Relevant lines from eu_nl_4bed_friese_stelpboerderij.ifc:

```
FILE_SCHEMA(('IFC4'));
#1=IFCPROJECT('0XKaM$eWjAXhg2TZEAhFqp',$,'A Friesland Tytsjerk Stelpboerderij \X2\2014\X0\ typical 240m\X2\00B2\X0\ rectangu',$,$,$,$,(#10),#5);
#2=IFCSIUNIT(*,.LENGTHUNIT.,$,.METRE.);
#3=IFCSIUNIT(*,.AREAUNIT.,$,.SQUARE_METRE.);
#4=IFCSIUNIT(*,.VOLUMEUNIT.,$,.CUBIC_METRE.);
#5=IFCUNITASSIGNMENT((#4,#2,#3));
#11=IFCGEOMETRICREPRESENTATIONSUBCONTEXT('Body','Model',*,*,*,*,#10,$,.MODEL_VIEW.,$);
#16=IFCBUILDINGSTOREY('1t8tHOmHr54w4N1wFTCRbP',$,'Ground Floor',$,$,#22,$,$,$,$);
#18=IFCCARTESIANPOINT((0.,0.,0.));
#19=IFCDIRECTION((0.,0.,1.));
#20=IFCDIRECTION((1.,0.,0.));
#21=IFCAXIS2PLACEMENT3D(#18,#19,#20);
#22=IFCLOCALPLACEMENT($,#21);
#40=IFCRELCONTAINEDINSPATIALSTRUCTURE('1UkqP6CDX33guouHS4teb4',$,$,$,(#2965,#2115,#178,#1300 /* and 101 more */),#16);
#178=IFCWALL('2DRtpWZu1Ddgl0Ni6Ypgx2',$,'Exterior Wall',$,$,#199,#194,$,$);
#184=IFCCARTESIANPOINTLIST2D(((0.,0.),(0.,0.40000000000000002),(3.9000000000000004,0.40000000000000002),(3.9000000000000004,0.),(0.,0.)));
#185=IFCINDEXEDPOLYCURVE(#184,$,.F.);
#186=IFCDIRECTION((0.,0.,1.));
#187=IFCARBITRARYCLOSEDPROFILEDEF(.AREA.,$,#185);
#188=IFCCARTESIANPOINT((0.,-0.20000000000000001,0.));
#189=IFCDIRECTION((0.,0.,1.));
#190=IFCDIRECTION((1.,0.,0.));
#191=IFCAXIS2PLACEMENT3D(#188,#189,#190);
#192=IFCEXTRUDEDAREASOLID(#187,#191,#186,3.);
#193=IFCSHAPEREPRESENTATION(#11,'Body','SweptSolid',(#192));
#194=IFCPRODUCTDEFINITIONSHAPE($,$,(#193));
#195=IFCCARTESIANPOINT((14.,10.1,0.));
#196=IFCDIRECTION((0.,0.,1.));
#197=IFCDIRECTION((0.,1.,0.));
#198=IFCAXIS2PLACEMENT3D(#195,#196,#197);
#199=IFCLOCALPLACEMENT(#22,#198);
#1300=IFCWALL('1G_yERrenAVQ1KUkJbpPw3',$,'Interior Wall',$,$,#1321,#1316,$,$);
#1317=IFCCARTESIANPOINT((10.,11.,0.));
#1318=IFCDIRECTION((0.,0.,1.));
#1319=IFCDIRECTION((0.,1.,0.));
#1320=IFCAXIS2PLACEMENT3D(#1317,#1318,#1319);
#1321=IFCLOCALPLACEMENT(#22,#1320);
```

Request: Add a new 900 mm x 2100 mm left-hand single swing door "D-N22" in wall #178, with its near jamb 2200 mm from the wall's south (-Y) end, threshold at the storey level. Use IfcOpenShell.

```python
import numpy as np
import ifcopenshell
import ifcopenshell.api.feature
import ifcopenshell.api.geometry
import ifcopenshell.api.root
import ifcopenshell.api.spatial
import ifcopenshell.geom
import ifcopenshell.util.element
import ifcopenshell.util.placement
import ifcopenshell.util.representation
import ifcopenshell.util.shape
import ifcopenshell.util.unit

model = ifcopenshell.open("eu_nl_4bed_friese_stelpboerderij.ifc")
unit_scale = ifcopenshell.util.unit.calculate_unit_scale(model)
settings = ifcopenshell.geom.settings()


def volume(element):
    """Net volume in cubic metres, openings subtracted."""
    shape = ifcopenshell.geom.create_shape(settings, element)
    return ifcopenshell.util.shape.get_volume(shape.geometry)


wall = model.by_guid("2DRtpWZu1Ddgl0Ni6Ypgx2")
storey = ifcopenshell.util.element.get_container(wall, ifc_class="IfcBuildingStorey")
context = ifcopenshell.util.representation.get_context(model, "Model", "Body", "MODEL_VIEW")
before = volume(wall)

width, height, from_end, sill = 0.9, 2.1, 2.2, 0.0  # metres

# The wall runs along its own X axis, and the end named is its -X end.
wall_shape = ifcopenshell.geom.create_shape(settings, wall)
x, y, z = ifcopenshell.util.shape.get_vertices(wall_shape.geometry).T
start = x.min() + from_end
face, thickness = float(y.min()), float(y.max() - y.min())
wall_matrix = ifcopenshell.util.placement.get_local_placement(wall.ObjectPlacement)
level = ifcopenshell.util.placement.get_local_placement(storey.ObjectPlacement)[2, 3]


def in_wall(x, y):
    """Placement at x, y metres in the wall's axes, at sill height."""
    matrix = wall_matrix.copy()
    matrix[:, 3] = wall_matrix @ np.array([x / unit_scale, y / unit_scale, 0.0, 1.0])
    matrix[2, 3] = level + sill / unit_scale
    return matrix


# Opening: a box that overshoots both wall faces by 50 mm.
opening = ifcopenshell.api.root.create_entity(model, ifc_class="IfcOpeningElement", predefined_type="OPENING")
box = ifcopenshell.api.geometry.add_wall_representation(
    model, context=context, length=width, height=height, thickness=thickness + 0.1
)
ifcopenshell.api.geometry.assign_representation(model, product=opening, representation=box)
ifcopenshell.api.geometry.edit_object_placement(model, product=opening, matrix=in_wall(start, face - 0.05), is_si=False)
ifcopenshell.api.feature.add_feature(model, feature=opening, element=wall)

door = ifcopenshell.api.root.create_entity(model, ifc_class="IfcDoor", name="D-N22", predefined_type="DOOR")
door.OverallWidth, door.OverallHeight = width / unit_scale, height / unit_scale
door.OperationType = "SINGLE_SWING_LEFT"
body = ifcopenshell.api.geometry.add_door_representation(
    model,
    context=context,
    overall_width=door.OverallWidth,
    overall_height=door.OverallHeight,
    operation_type="SINGLE_SWING_LEFT",
    lining_properties={"LiningDepth": thickness / unit_scale, "ThresholdDepth": thickness / unit_scale},
)
ifcopenshell.api.geometry.assign_representation(model, product=door, representation=body)
ifcopenshell.api.spatial.assign_container(model, products=[door], relating_structure=storey)
ifcopenshell.api.feature.add_filling(model, opening=opening, element=door)

# The lining spans the wall, so the door starts at the wall face.
ifcopenshell.api.geometry.edit_object_placement(model, product=door, matrix=in_wall(start, face), is_si=False)

after = volume(wall)

print(f"wall volume {before:.3f} -> {after:.3f} m3")

model.write("eu_nl_4bed_friese_stelpboerderij_edited.ifc")
```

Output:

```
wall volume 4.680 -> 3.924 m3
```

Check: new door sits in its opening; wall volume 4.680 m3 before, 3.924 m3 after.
